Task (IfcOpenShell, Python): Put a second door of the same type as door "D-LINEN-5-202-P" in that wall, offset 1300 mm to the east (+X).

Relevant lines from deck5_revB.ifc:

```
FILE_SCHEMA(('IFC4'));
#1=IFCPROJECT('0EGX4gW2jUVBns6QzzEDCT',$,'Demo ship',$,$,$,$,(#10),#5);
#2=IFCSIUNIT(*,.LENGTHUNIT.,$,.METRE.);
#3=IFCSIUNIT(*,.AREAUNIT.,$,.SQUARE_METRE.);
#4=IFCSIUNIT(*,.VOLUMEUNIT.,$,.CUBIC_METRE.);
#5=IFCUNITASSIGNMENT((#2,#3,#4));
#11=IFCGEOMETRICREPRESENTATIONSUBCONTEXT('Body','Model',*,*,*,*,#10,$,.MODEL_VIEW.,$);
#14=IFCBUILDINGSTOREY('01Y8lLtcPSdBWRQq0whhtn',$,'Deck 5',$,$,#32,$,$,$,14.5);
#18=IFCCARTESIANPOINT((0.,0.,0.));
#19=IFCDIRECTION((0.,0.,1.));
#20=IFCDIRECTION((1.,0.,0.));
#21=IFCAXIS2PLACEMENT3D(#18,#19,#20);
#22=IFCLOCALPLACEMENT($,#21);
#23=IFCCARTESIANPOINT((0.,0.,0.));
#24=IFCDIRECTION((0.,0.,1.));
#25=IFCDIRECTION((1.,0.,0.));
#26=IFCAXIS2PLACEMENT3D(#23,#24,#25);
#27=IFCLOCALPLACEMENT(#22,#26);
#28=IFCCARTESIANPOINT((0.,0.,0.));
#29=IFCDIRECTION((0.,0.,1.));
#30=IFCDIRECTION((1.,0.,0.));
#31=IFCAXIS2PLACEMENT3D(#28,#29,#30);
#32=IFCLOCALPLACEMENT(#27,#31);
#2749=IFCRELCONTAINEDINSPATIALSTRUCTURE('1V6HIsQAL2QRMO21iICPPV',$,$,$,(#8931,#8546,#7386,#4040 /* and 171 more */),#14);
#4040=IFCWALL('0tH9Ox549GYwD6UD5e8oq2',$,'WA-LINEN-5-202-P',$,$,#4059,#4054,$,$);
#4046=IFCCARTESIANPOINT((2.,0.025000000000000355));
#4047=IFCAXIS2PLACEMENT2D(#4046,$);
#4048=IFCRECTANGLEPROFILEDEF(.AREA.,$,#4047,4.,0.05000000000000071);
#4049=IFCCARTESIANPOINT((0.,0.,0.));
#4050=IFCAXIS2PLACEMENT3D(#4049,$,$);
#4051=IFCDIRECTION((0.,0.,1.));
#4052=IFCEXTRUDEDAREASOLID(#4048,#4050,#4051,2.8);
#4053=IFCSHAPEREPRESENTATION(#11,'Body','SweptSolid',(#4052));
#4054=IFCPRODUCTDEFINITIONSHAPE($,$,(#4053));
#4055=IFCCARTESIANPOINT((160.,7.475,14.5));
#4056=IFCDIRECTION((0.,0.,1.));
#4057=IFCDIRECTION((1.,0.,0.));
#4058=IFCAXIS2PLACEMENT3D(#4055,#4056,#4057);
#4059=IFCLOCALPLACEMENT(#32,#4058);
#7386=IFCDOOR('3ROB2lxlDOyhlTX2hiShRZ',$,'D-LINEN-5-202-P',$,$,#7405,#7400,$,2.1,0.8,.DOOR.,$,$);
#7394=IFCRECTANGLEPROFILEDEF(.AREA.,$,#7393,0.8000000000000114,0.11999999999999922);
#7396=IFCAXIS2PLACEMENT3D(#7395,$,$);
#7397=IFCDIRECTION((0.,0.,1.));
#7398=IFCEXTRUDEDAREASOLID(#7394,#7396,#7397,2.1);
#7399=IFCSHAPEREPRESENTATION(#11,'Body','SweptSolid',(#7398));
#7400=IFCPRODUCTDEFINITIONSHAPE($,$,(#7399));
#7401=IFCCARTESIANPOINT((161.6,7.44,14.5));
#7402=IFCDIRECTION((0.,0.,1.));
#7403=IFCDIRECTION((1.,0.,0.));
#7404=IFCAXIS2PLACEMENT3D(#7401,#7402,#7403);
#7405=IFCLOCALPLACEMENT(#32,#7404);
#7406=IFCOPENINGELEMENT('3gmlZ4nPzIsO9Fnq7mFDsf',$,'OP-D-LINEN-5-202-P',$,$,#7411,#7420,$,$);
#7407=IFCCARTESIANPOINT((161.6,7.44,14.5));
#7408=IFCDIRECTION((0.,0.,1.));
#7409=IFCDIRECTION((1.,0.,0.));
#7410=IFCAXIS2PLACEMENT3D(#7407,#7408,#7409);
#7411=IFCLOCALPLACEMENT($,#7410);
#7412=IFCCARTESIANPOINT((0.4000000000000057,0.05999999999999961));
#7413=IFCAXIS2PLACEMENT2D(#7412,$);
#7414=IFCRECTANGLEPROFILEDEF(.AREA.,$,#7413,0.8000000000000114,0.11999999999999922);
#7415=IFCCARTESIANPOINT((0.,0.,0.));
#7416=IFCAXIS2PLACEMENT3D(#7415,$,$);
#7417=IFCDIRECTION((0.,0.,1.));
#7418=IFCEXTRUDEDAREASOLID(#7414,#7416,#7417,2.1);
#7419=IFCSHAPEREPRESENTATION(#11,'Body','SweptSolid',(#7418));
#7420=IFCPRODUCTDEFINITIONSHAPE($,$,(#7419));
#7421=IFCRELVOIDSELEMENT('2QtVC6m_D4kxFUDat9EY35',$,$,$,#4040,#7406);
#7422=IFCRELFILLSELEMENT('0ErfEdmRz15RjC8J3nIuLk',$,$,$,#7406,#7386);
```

```python
import ifcopenshell
import ifcopenshell.api.feature
import ifcopenshell.api.geometry
import ifcopenshell.api.root
import ifcopenshell.geom
import ifcopenshell.util.element
import ifcopenshell.util.placement
import ifcopenshell.util.shape

model = ifcopenshell.open("deck5_revB.ifc")
settings = ifcopenshell.geom.settings()


def volume(element):
    """Net volume in cubic metres, openings subtracted."""
    shape = ifcopenshell.geom.create_shape(settings, element)
    return ifcopenshell.util.shape.get_volume(shape.geometry)


door = model.by_guid("3ROB2lxlDOyhlTX2hiShRZ")
opening = door.FillsVoids[0].RelatingOpeningElement
wall = opening.VoidsElements[0].RelatingBuildingElement
before = volume(wall)
shift = ifcopenshell.util.placement.get_local_placement(wall.ObjectPlacement)[:3, 0] * 1.3

# copy_class copies the void relationship, type, container and properties, but no geometry.
new_opening = ifcopenshell.api.root.copy_class(model, product=opening)
new_opening.Representation = ifcopenshell.util.element.copy_deep(
    model, opening.Representation, exclude=["IfcGeometricRepresentationContext", "IfcRepresentationMap"]
)
new_door = ifcopenshell.api.root.copy_class(model, product=door)
new_door.Representation = ifcopenshell.util.element.copy_deep(
    model, door.Representation, exclude=["IfcGeometricRepresentationContext", "IfcRepresentationMap"]
)
ifcopenshell.api.feature.add_filling(model, opening=new_opening, element=new_door)

for old, new in ((opening, new_opening), (door, new_door)):
    matrix = ifcopenshell.util.placement.get_local_placement(old.ObjectPlacement)
    matrix[:3, 3] += shift
    ifcopenshell.api.geometry.edit_object_placement(model, product=new, matrix=matrix, is_si=False)

after = volume(wall)

print(f"wall volume {before:.3f} -> {after:.3f} m3")

model.write("deck5_revB_rev.ifc")
```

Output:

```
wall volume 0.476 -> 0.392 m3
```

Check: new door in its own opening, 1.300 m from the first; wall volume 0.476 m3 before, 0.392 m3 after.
